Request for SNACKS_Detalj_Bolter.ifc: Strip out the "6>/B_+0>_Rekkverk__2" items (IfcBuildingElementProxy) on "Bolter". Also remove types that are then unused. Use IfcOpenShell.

First a look at what the model holds.

```python
import ifcopenshell
import ifcopenshell.util.element

model = ifcopenshell.open("SNACKS_Detalj_Bolter.ifc")
print(model.schema)
storey = next(s for s in model.by_type("IfcBuildingStorey") if s.Name == "Bolter")
proxies = [e for e in ifcopenshell.util.element.get_decomposition(storey) if e.is_a("IfcBuildingElementProxy")]
seen = {}
for e in proxies:
    element_type = ifcopenshell.util.element.get_type(e)
    name = element_type.Name if element_type not in (None, e) else None
    seen[name] = seen.get(name, 0) + 1
for name, count in sorted(seen.items(), key=str):
    print(count, "x", name)
```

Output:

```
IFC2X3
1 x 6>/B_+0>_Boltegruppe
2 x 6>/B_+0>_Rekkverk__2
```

```python
import ifcopenshell
import ifcopenshell.api.root
import ifcopenshell.util.element

model = ifcopenshell.open("SNACKS_Detalj_Bolter.ifc")

storey = next(s for s in model.by_type("IfcBuildingStorey") if s.Name == "Bolter")
proxies = [e for e in ifcopenshell.util.element.get_decomposition(storey) if e.is_a("IfcBuildingElementProxy")]
targets = [e for e in proxies if (t := ifcopenshell.util.element.get_type(e)) not in (None, e) and t.Name == "6>/B_+0>_Rekkverk__2"]
types = {ifcopenshell.util.element.get_type(e) for e in targets} - {None, *targets}

for e in targets:
    ifcopenshell.api.root.remove_product(model, product=e)
print(len(targets), "removed")

unused = [t for t in types if not ifcopenshell.util.element.get_types(t)]
for t in unused:
    ifcopenshell.api.root.remove_product(model, product=t)
print(len(unused), "unused types removed")

model.write("SNACKS_Detalj_Bolter_rev.ifc")
```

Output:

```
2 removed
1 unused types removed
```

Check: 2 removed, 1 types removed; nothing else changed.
